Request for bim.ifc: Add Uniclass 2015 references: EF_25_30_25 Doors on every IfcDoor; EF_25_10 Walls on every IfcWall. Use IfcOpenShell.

First a look at what the model holds.

```python
import ifcopenshell

model = ifcopenshell.open("bim.ifc")
print(model.schema)
print("classifications:", [c.Name for c in model.by_type("IfcClassification")])
for ifc_class in ("IfcDoor", "IfcRoof", "IfcStair", "IfcWall", "IfcWindow"):
    print(ifc_class, len(model.by_type(ifc_class)))
```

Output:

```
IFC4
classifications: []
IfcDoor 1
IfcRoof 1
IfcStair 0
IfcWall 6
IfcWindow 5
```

```python
import ifcopenshell
import ifcopenshell.api.classification

model = ifcopenshell.open("bim.ifc")

system = ifcopenshell.api.classification.add_classification(model, classification="Uniclass 2015")

codes = {
    "IfcDoor": ("EF_25_30_25", "Doors"),
    "IfcWall": ("EF_25_10", "Walls"),
}
for ifc_class, (code, name) in codes.items():
    products = model.by_type(ifc_class)
    ifcopenshell.api.classification.add_reference(
        model, products=products, classification=system, identification=code, name=name
    )
    print(code, len(products))

model.write("bim-out.ifc")
```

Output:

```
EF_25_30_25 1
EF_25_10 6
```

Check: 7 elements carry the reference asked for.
